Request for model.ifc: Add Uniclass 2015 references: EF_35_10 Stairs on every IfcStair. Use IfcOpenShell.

First a look at what the model holds.

```python
import ifcopenshell

model = ifcopenshell.open("model.ifc")
print(model.schema)
print("classifications:", [c.Name for c in model.by_type("IfcClassification")])
for ifc_class in ("IfcDoor", "IfcRoof", "IfcStair", "IfcWall", "IfcWindow"):
    print(ifc_class, len(model.by_type(ifc_class)))
```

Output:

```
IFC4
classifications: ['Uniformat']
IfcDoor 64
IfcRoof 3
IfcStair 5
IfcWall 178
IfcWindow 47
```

```python
import ifcopenshell
import ifcopenshell.api.classification

model = ifcopenshell.open("model.ifc")

system = ifcopenshell.api.classification.add_classification(model, classification="Uniclass 2015")

codes = {
    "IfcStair": ("EF_35_10", "Stairs"),
}
for ifc_class, (code, name) in codes.items():
    products = model.by_type(ifc_class)
    ifcopenshell.api.classification.add_reference(
        model, products=products, classification=system, identification=code, name=name
    )
    print(code, len(products))

model.write("model_edited.ifc")
```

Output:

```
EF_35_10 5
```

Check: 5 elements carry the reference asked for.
